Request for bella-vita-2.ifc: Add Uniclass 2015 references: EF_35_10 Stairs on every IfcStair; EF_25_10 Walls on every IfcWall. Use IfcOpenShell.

First a look at what the model holds.

```python
import ifcopenshell

model = ifcopenshell.open("bella-vita-2.ifc")
print(model.schema)
print("classifications:", [c.Name for c in model.by_type("IfcClassification")])
for ifc_class in ("IfcDoor", "IfcRoof", "IfcStair", "IfcWall", "IfcWindow"):
    print(ifc_class, len(model.by_type(ifc_class)))
```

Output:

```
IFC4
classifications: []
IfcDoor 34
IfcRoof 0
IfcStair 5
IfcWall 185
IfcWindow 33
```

```python
import ifcopenshell
import ifcopenshell.api.classification

model = ifcopenshell.open("bella-vita-2.ifc")

system = ifcopenshell.api.classification.add_classification(model, classification="Uniclass 2015")

codes = {
    "IfcStair": ("EF_35_10", "Stairs"),
    "IfcWall": ("EF_25_10", "Walls"),
}
for ifc_class, (code, name) in codes.items():
    products = model.by_type(ifc_class)
    ifcopenshell.api.classification.add_reference(
        model, products=products, classification=system, identification=code, name=name
    )
    print(code, len(products))

model.write("bella-vita-2_v2.ifc")
```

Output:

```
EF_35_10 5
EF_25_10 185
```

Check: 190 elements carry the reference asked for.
